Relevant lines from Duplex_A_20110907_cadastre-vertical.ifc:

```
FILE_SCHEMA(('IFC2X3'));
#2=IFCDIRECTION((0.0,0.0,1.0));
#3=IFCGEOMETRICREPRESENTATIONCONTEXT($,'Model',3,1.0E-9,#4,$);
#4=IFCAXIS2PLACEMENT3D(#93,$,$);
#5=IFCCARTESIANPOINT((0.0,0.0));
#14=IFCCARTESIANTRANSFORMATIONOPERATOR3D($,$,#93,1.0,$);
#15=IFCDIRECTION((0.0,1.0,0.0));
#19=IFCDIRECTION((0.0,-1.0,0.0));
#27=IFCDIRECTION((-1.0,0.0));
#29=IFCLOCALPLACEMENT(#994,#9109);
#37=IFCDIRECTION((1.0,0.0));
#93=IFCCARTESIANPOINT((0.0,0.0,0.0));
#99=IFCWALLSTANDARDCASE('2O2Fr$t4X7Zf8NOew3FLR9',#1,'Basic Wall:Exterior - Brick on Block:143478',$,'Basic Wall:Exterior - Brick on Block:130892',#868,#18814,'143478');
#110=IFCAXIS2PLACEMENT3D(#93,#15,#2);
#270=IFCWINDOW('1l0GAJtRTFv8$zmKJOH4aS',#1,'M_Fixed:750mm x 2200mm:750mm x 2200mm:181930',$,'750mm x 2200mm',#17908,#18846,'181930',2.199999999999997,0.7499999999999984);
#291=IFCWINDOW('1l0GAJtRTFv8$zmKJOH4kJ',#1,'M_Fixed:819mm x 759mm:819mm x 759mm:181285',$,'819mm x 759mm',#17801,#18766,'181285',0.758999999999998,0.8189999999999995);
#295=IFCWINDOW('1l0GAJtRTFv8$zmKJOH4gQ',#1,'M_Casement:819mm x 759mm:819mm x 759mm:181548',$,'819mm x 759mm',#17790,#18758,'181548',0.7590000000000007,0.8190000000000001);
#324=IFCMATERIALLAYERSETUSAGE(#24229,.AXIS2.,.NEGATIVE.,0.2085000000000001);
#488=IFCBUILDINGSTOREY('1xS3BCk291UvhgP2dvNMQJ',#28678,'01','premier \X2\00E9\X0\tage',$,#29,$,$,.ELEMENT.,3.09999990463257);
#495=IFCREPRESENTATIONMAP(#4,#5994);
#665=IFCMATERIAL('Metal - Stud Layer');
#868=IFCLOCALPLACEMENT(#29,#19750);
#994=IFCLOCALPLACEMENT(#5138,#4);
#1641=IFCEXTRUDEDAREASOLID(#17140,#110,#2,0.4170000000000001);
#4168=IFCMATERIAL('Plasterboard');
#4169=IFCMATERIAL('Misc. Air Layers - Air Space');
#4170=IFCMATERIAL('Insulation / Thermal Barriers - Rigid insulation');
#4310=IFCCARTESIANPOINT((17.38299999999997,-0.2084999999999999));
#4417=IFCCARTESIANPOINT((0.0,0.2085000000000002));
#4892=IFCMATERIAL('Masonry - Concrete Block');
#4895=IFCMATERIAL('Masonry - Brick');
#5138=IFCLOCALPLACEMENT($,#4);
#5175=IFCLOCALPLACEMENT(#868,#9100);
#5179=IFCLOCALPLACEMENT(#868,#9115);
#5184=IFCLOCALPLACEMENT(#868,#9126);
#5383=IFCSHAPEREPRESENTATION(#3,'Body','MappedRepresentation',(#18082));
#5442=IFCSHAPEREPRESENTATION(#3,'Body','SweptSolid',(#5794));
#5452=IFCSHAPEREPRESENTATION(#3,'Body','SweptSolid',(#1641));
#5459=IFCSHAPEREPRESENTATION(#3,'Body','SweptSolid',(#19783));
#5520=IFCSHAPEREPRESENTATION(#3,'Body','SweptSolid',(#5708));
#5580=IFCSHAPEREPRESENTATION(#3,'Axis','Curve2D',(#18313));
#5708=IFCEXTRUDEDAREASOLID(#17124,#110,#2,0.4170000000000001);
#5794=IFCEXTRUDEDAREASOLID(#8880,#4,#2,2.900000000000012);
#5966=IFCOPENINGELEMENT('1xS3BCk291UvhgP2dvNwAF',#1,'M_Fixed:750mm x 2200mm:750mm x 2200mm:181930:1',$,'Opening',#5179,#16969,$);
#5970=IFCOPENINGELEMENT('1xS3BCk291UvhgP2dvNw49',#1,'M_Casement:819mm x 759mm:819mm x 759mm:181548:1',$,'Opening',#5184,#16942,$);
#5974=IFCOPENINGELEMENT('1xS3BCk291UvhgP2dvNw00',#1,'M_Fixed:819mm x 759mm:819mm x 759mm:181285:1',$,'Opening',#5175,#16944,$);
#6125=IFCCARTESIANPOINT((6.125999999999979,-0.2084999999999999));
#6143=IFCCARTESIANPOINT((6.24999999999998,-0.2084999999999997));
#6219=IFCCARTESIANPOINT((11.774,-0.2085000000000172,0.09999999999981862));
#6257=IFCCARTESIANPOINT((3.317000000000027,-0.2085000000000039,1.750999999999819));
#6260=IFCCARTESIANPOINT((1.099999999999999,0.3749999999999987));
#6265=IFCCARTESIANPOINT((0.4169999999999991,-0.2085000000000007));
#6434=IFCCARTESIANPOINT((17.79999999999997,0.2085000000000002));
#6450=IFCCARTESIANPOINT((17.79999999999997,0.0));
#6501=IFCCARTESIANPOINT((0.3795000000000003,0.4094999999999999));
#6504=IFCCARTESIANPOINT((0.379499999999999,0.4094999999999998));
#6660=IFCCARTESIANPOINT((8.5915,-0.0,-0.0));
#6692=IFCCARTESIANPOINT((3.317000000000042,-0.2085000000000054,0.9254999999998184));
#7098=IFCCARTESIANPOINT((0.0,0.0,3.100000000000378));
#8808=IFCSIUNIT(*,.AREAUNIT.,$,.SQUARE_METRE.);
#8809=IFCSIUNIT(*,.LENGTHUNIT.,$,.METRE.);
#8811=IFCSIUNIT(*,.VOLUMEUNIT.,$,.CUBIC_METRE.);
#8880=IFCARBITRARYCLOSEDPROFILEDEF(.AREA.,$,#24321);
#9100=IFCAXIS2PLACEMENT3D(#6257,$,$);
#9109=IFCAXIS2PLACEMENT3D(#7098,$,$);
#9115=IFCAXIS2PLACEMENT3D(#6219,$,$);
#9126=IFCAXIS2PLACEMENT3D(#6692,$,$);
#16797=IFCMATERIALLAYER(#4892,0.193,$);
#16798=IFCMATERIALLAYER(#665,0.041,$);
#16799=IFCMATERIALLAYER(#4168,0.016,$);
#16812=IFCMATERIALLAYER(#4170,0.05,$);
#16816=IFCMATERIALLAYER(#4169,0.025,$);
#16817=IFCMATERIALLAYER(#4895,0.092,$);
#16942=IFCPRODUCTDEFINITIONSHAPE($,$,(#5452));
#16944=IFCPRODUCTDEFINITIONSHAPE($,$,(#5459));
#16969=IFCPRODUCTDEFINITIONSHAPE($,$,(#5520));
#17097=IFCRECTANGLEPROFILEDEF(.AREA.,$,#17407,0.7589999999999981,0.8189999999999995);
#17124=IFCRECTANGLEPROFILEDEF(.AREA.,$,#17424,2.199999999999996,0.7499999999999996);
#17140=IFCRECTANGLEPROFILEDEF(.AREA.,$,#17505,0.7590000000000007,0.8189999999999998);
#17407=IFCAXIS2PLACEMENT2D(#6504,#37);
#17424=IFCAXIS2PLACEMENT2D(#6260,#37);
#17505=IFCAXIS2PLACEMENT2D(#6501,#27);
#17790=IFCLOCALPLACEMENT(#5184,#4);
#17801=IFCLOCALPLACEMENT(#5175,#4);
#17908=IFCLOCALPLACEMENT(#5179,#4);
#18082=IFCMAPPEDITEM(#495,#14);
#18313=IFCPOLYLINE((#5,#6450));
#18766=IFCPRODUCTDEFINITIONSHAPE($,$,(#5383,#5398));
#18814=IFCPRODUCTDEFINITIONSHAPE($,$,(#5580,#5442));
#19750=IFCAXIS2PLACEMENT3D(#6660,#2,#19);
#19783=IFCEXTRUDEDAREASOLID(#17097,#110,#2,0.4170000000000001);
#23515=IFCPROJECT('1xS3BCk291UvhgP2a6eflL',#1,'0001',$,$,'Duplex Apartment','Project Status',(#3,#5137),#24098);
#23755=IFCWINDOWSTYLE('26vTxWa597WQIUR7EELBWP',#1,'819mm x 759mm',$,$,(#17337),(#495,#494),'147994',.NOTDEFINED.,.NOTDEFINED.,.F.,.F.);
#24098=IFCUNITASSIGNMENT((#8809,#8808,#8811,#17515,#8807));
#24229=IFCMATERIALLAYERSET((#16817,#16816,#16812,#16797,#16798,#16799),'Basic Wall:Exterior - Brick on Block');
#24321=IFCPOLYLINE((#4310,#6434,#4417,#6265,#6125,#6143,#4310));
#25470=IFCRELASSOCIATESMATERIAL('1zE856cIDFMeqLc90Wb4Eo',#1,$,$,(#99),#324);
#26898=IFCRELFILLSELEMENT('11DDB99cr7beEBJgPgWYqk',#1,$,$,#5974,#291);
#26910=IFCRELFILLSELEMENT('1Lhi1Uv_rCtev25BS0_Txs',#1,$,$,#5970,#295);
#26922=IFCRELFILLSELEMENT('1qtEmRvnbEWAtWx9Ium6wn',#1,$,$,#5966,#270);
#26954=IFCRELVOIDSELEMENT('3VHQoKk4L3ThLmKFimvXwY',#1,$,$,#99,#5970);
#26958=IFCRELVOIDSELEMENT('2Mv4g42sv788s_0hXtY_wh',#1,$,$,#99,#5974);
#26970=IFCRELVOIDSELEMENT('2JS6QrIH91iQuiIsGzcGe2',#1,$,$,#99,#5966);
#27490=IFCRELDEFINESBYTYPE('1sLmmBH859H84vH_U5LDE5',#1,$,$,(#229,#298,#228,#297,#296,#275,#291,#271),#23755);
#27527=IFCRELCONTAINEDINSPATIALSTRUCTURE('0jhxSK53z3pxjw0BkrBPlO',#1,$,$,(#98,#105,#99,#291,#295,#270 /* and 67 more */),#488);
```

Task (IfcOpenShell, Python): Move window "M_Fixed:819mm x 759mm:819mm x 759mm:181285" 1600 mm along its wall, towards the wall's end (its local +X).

```python
import ifcopenshell
import ifcopenshell.api.geometry
import ifcopenshell.util.placement
import ifcopenshell.util.unit

model = ifcopenshell.open("Duplex_A_20110907_cadastre-vertical.ifc")
unit_scale = ifcopenshell.util.unit.calculate_unit_scale(model)

window = model.by_id(291)
opening = window.FillsVoids[0].RelatingOpeningElement
wall = opening.VoidsElements[0].RelatingBuildingElement

wall_matrix = ifcopenshell.util.placement.get_local_placement(wall.ObjectPlacement)
shift = wall_matrix[:3, 0] * 1.6 / unit_scale
before = ifcopenshell.util.placement.get_local_placement(window.ObjectPlacement)[:3, 3].copy()

# The window is placed relative to its opening, so it follows when the opening moves.
matrix = ifcopenshell.util.placement.get_local_placement(opening.ObjectPlacement)
matrix[:3, 3] += shift
ifcopenshell.api.geometry.edit_object_placement(
    model, product=opening, matrix=matrix, is_si=False, should_transform_children=True
)

after = ifcopenshell.util.placement.get_local_placement(window.ObjectPlacement)[:3, 3]
print("window moved by", (after - before).round(3) + 0.0)

model.write("Duplex_A_20110907_cadastre-vertical_v2.ifc")
```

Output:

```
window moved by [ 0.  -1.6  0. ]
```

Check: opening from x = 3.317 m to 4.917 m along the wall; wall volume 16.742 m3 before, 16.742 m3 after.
